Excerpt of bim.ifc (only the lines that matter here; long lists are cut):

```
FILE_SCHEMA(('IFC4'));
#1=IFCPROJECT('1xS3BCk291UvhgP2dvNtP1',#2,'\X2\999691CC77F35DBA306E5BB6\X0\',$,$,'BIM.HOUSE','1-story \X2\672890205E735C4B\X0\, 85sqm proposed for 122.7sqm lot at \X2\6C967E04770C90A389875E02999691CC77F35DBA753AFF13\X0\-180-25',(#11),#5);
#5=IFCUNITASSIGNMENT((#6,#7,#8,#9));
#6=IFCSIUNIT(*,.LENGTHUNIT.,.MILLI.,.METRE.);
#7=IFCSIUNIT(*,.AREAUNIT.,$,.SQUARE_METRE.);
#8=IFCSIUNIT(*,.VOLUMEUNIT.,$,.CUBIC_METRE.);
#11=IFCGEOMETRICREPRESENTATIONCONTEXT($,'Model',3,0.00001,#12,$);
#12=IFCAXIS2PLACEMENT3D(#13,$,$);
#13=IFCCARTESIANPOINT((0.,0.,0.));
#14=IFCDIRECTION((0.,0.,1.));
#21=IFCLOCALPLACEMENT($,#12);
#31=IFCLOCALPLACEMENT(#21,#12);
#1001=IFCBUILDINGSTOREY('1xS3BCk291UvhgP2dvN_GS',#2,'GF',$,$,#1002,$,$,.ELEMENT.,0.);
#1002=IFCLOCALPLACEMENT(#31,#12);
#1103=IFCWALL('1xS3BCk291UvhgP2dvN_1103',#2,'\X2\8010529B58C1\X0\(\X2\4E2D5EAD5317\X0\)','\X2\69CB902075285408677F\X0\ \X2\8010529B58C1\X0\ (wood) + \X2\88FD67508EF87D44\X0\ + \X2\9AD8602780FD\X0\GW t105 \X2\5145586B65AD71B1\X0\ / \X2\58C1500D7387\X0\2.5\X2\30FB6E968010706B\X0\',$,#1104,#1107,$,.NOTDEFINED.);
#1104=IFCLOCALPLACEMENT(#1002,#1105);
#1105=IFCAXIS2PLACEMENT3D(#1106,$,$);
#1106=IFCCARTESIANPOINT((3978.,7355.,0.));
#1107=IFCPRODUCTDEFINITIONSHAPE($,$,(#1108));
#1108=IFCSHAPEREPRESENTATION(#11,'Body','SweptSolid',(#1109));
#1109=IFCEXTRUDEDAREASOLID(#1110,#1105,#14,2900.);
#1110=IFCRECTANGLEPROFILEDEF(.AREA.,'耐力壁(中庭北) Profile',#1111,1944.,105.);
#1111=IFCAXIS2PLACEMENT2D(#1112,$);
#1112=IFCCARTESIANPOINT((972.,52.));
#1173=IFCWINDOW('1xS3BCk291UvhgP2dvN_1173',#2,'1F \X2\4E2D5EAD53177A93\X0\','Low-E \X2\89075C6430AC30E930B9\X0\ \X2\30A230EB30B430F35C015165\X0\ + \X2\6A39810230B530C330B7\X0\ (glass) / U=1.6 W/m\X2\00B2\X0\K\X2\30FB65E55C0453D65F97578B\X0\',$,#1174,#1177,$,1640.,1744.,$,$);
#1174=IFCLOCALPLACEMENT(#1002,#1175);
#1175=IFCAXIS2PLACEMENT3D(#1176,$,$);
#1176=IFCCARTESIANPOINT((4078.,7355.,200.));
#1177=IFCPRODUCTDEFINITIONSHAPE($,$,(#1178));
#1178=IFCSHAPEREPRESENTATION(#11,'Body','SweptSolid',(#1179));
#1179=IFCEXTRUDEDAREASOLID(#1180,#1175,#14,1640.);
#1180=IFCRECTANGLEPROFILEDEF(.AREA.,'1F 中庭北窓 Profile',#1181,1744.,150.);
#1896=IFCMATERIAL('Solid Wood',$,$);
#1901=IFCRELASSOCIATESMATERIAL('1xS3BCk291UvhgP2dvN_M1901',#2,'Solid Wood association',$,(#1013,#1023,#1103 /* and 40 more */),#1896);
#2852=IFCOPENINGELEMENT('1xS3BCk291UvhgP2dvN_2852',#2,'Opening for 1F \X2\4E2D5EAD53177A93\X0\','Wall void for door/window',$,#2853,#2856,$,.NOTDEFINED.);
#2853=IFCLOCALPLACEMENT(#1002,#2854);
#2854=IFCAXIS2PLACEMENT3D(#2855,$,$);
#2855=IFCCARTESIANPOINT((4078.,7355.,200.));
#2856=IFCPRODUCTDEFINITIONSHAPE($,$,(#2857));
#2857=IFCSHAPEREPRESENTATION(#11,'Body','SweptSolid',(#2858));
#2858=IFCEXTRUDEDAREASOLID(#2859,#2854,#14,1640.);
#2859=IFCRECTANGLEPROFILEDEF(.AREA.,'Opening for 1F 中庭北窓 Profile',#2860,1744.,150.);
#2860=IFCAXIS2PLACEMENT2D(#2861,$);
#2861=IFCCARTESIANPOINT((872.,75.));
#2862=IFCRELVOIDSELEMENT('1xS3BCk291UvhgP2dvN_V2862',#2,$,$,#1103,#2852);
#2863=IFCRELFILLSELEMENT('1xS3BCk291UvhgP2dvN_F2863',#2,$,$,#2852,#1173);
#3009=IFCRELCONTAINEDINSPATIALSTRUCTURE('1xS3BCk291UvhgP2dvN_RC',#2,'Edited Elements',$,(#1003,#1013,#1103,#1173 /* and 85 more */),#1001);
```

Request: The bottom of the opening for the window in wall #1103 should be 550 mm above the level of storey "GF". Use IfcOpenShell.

```python
import numpy as np
import ifcopenshell
import ifcopenshell.api.geometry
import ifcopenshell.geom
import ifcopenshell.util.element
import ifcopenshell.util.placement
import ifcopenshell.util.shape
import ifcopenshell.util.unit

model = ifcopenshell.open("bim.ifc")
unit_scale = ifcopenshell.util.unit.calculate_unit_scale(model)

window = model.by_guid("1xS3BCk291UvhgP2dvN_1173")
opening = window.FillsVoids[0].RelatingOpeningElement
storey = ifcopenshell.util.element.get_container(window, ifc_class="IfcBuildingStorey")
level = ifcopenshell.util.placement.get_local_placement(storey.ObjectPlacement)[2, 3]

# The opening's origin need not be at the sill, so measure its lowest point.
shape = ifcopenshell.geom.create_shape(ifcopenshell.geom.settings(), opening)
bottom = ifcopenshell.util.shape.get_shape_bottom_elevation(shape, shape.geometry) / unit_scale
dz = level + 550.0 - bottom

shift = np.array([0.0, 0.0, dz])
# The window is not placed relative to its opening, so move both.
for product in (opening, window):
    matrix = ifcopenshell.util.placement.get_local_placement(product.ObjectPlacement)
    matrix[:3, 3] += shift
    ifcopenshell.api.geometry.edit_object_placement(model, product=product, matrix=matrix, is_si=False)

print(f"moved by {dz * unit_scale:+.3f} m")

model.write("bim_rev.ifc")
```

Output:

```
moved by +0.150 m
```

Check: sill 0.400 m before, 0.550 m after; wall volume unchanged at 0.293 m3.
